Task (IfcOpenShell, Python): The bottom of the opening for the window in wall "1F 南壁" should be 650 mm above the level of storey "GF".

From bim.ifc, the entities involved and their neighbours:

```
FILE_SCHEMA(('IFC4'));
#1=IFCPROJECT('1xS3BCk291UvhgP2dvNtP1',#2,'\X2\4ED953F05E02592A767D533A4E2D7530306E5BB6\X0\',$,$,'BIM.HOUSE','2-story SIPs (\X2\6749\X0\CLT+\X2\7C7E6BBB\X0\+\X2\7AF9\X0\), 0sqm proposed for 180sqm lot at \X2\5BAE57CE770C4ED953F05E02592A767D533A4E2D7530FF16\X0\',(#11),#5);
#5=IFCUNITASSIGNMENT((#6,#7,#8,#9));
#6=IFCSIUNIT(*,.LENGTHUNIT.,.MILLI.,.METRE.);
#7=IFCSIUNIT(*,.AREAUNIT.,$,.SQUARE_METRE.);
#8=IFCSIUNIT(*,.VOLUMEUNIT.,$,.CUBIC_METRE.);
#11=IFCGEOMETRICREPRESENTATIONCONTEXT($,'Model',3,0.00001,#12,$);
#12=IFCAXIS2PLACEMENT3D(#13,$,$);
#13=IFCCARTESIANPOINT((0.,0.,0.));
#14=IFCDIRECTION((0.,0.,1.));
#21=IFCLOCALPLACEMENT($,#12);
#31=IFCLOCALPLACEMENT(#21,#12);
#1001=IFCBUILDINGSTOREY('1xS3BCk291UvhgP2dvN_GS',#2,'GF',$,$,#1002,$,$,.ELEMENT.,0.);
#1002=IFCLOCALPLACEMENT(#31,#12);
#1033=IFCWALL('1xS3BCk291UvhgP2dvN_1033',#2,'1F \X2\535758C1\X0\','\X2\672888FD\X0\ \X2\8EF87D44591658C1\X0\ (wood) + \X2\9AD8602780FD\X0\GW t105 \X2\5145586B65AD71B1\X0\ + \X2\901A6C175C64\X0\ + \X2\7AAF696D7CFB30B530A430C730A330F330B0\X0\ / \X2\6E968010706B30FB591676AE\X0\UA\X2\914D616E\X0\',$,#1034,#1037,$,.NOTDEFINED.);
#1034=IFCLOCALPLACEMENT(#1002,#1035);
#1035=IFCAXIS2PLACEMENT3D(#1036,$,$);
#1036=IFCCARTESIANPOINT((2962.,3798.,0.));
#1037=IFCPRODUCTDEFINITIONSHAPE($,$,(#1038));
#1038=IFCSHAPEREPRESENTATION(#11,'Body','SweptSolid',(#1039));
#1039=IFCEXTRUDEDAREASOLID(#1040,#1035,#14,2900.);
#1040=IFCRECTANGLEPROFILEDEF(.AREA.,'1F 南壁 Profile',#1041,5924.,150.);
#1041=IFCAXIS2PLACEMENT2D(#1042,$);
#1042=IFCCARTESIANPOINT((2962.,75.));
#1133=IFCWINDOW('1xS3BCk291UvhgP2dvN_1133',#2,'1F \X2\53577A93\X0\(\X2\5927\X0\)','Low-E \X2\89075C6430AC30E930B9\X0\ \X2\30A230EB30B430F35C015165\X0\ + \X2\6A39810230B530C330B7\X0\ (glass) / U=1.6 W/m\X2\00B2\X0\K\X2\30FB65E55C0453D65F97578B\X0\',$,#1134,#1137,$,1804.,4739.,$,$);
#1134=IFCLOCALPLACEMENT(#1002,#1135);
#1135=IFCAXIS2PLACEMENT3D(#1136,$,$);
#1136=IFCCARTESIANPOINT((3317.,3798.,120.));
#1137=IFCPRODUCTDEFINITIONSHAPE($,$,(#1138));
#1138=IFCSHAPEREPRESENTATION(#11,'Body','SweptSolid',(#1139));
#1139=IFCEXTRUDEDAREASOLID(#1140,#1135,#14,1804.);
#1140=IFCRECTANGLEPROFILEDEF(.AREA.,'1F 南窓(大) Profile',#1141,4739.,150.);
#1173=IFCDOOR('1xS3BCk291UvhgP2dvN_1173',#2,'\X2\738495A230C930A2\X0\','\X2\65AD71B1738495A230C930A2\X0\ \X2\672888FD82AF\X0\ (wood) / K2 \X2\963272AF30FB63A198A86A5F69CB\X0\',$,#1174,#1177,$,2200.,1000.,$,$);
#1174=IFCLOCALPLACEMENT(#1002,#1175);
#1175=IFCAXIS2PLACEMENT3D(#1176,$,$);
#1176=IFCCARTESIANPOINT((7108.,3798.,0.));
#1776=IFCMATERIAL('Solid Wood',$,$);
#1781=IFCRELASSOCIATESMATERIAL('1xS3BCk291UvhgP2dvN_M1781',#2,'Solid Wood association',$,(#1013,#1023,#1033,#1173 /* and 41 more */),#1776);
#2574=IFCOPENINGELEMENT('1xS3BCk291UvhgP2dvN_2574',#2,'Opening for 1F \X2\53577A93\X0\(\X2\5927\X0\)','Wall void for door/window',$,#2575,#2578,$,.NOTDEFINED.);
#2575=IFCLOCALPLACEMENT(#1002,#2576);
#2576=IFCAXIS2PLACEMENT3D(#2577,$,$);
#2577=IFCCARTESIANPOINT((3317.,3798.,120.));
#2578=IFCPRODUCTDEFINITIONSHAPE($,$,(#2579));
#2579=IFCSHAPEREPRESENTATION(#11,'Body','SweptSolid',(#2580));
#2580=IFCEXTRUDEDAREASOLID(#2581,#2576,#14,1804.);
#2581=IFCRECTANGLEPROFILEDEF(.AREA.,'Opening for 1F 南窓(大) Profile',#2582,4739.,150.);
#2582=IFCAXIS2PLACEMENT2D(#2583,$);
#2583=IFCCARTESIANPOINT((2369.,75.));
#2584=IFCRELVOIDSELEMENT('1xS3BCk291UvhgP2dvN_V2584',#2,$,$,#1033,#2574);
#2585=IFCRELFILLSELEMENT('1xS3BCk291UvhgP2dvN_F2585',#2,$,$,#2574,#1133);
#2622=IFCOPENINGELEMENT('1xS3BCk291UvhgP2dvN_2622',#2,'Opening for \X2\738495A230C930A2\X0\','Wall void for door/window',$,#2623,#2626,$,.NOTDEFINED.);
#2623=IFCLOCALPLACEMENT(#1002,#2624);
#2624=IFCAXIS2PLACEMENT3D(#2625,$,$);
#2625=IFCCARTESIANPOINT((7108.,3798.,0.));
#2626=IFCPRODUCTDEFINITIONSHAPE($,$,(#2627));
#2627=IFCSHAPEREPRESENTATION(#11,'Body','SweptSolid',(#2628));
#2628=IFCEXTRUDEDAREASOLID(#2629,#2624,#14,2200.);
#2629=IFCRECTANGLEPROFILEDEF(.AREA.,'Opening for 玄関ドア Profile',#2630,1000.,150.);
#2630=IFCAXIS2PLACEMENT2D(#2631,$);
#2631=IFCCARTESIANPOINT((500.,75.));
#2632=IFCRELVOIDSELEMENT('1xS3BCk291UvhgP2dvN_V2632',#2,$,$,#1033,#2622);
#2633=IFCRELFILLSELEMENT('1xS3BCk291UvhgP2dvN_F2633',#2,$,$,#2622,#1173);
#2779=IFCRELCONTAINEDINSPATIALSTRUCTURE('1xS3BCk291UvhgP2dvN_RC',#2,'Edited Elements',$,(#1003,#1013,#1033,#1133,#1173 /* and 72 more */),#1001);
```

```python
import numpy as np
import ifcopenshell
import ifcopenshell.api.geometry
import ifcopenshell.geom
import ifcopenshell.util.element
import ifcopenshell.util.placement
import ifcopenshell.util.shape
import ifcopenshell.util.unit

model = ifcopenshell.open("bim.ifc")
unit_scale = ifcopenshell.util.unit.calculate_unit_scale(model)

window = model.by_guid("1xS3BCk291UvhgP2dvN_1133")
opening = window.FillsVoids[0].RelatingOpeningElement
storey = ifcopenshell.util.element.get_container(window, ifc_class="IfcBuildingStorey")
level = ifcopenshell.util.placement.get_local_placement(storey.ObjectPlacement)[2, 3]

# The opening's origin need not be at the sill, so measure its lowest point.
shape = ifcopenshell.geom.create_shape(ifcopenshell.geom.settings(), opening)
bottom = ifcopenshell.util.shape.get_shape_bottom_elevation(shape, shape.geometry) / unit_scale
dz = level + 0.65 / unit_scale - bottom

shift = np.array([0.0, 0.0, dz])
# The window is not placed relative to its opening, so move both.
for product in (opening, window):
    matrix = ifcopenshell.util.placement.get_local_placement(product.ObjectPlacement)
    matrix[:3, 3] += shift
    ifcopenshell.api.geometry.edit_object_placement(model, product=product, matrix=matrix, is_si=False)

print(f"moved by {dz * unit_scale:+.3f} m")

model.write("bim_v2.ifc")
```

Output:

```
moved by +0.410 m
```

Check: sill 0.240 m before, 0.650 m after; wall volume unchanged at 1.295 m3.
